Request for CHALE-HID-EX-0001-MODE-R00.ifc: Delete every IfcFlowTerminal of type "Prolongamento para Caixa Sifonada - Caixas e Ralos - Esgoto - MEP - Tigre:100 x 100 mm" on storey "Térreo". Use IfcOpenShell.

First a look at what the model holds.

```python
import ifcopenshell
import ifcopenshell.util.element

model = ifcopenshell.open("CHALE-HID-EX-0001-MODE-R00.ifc")
print(model.schema)
storey = next(s for s in model.by_type("IfcBuildingStorey") if s.Name == "Térreo")
terminals = [e for e in ifcopenshell.util.element.get_decomposition(storey) if e.is_a("IfcFlowTerminal")]
seen = {}
for e in terminals:
    element_type = ifcopenshell.util.element.get_type(e)
    name = element_type.Name if element_type not in (None, e) else None
    seen[name] = seen.get(name, 0) + 1
for name, count in sorted(seen.items(), key=str):
    print(count, "x", name)
```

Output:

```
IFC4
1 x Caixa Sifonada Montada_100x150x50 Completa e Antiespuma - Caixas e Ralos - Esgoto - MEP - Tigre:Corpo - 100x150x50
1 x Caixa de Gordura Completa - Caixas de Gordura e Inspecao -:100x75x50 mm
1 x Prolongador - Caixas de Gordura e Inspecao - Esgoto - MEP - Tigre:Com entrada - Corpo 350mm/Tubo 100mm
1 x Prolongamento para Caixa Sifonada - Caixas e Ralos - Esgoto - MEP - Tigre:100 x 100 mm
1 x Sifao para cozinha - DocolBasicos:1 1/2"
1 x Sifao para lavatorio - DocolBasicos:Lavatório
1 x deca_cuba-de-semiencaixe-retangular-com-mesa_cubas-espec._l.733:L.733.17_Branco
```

```python
import ifcopenshell
import ifcopenshell.api.root
import ifcopenshell.util.element

model = ifcopenshell.open("CHALE-HID-EX-0001-MODE-R00.ifc")

storey = next(s for s in model.by_type("IfcBuildingStorey") if s.Name == "Térreo")
terminals = [e for e in ifcopenshell.util.element.get_decomposition(storey) if e.is_a("IfcFlowTerminal")]
targets = [e for e in terminals if (t := ifcopenshell.util.element.get_type(e)) not in (None, e) and t.Name == "Prolongamento para Caixa Sifonada - Caixas e Ralos - Esgoto - MEP - Tigre:100 x 100 mm"]

for e in targets:
    ifcopenshell.api.root.remove_product(model, product=e)
print(len(targets), "removed")

model.write("CHALE-HID-EX-0001-MODE-R00_edited.ifc")
```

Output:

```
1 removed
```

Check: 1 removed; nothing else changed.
